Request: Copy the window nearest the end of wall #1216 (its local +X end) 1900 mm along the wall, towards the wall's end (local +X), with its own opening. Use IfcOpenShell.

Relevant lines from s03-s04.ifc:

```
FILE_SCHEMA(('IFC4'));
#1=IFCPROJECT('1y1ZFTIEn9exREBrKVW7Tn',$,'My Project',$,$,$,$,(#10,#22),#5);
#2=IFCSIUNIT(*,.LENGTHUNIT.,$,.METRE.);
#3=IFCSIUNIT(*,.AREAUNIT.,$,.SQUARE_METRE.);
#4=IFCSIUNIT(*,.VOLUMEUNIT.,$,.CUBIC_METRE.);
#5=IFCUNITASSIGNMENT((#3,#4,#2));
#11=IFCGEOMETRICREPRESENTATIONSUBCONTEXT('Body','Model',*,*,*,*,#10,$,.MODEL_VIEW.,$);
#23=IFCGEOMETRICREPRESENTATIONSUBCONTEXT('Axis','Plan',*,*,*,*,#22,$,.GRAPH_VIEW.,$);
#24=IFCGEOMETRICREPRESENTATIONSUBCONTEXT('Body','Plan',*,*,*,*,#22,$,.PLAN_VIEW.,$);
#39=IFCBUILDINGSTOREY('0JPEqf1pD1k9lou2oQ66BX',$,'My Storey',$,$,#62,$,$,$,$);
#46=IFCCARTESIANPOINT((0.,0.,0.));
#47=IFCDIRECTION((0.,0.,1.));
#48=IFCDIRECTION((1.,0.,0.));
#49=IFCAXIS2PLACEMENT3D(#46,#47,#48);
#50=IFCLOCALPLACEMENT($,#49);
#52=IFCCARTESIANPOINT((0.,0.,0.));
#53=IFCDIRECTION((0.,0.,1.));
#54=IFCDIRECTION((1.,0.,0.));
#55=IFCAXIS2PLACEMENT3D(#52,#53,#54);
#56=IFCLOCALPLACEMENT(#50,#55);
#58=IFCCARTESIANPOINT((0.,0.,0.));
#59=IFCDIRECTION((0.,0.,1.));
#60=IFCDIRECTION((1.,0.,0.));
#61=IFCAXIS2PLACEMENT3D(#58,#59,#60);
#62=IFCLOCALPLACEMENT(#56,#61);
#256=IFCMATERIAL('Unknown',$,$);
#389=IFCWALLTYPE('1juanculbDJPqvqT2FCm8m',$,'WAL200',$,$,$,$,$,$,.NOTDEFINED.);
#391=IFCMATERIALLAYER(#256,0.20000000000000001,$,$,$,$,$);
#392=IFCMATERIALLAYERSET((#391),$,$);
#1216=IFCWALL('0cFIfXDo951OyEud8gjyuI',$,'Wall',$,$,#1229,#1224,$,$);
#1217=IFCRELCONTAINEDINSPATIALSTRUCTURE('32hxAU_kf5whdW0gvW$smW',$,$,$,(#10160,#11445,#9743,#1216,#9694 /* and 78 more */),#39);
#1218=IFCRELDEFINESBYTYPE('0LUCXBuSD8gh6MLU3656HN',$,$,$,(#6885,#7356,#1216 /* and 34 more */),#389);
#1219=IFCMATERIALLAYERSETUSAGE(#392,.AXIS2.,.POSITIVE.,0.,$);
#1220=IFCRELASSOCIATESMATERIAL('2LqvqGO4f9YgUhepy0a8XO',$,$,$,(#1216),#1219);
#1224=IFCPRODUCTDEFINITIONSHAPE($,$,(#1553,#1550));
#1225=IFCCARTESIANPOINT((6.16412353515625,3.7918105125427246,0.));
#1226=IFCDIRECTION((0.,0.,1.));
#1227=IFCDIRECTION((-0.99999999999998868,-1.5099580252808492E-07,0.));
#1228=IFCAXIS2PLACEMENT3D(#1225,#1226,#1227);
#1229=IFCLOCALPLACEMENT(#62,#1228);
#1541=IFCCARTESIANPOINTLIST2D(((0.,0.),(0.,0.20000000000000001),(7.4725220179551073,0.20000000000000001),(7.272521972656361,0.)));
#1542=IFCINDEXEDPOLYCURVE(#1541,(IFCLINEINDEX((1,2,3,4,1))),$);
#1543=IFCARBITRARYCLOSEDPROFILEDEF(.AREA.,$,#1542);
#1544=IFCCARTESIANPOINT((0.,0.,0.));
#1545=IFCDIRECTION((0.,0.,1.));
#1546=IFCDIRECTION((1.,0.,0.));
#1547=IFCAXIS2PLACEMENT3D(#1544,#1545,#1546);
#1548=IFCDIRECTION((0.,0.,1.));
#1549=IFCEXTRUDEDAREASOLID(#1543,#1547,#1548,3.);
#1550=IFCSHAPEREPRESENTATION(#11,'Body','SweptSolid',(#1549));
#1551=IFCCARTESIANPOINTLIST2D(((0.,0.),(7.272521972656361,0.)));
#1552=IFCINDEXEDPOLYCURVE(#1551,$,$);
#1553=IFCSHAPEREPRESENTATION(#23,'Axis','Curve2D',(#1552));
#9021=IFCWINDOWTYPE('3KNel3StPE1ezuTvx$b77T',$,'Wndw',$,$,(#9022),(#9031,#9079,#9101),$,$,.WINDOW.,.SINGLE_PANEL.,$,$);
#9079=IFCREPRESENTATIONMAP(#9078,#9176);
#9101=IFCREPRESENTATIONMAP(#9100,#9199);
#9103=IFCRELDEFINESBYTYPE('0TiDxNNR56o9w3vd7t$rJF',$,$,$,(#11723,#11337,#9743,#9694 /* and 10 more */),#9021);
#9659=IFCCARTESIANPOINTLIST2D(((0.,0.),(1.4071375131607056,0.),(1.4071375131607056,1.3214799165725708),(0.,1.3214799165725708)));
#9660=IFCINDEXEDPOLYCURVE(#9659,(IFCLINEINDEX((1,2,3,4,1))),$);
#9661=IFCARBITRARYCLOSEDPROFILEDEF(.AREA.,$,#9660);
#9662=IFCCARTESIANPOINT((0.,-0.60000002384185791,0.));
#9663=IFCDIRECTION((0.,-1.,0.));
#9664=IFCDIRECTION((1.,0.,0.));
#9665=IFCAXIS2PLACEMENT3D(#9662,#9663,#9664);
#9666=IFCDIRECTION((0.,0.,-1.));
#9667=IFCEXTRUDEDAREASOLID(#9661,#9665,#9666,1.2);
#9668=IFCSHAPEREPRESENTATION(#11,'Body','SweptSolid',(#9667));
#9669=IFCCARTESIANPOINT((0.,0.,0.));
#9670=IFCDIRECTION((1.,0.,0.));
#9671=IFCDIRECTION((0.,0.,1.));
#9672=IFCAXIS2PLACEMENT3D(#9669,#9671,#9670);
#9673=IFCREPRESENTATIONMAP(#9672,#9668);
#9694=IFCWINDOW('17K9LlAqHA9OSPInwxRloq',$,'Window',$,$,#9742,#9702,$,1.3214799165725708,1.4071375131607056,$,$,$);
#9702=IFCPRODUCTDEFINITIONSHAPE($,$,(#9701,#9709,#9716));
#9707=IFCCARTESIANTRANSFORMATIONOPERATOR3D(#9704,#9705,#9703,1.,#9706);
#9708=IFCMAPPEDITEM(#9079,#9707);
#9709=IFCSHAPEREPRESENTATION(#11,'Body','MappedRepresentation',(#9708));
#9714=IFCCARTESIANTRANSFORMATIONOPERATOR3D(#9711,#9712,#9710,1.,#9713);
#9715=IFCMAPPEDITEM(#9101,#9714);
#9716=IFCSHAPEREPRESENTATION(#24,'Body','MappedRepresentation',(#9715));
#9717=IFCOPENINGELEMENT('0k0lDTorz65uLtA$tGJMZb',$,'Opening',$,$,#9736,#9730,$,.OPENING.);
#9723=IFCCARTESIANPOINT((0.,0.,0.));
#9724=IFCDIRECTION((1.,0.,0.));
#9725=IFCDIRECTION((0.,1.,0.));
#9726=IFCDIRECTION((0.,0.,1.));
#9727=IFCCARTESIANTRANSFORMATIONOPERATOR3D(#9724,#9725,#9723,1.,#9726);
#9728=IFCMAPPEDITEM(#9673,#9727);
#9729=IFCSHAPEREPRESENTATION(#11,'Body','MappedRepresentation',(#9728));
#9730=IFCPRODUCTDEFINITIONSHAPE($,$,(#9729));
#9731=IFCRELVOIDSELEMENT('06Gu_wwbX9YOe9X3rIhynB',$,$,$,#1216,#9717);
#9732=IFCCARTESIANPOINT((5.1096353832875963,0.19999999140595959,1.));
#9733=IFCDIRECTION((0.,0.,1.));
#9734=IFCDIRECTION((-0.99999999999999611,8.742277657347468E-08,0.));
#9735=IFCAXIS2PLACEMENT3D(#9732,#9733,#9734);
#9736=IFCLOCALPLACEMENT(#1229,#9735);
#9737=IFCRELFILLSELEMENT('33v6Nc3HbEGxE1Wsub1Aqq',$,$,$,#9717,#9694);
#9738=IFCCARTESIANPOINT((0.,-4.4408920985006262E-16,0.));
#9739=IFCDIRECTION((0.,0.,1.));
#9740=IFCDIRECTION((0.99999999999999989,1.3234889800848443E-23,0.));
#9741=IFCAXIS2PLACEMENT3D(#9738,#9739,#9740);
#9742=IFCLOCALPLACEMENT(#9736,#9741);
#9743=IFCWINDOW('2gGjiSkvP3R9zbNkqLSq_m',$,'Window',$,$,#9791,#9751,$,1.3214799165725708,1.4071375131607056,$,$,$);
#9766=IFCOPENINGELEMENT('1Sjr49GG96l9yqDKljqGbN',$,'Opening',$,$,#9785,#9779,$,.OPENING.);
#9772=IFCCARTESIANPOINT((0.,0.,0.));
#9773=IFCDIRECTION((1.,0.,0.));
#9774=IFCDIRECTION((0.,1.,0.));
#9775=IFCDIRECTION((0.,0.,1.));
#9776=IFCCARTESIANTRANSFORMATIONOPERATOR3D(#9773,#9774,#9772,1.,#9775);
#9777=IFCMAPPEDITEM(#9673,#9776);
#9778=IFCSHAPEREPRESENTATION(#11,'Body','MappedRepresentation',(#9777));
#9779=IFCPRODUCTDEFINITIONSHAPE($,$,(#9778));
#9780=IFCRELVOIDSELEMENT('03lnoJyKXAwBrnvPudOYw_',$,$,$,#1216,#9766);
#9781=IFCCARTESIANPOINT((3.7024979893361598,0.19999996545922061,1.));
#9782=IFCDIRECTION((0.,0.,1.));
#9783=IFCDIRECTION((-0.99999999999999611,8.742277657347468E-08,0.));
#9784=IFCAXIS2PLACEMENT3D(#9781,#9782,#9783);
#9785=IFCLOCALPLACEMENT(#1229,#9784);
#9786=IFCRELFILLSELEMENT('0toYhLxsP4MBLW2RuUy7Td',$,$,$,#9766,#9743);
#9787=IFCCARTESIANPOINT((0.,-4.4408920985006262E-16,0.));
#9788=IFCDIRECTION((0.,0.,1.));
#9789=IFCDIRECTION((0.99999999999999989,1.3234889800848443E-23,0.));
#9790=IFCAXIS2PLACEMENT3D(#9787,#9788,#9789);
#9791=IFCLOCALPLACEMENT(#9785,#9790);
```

```python
import ifcopenshell
import ifcopenshell.api.feature
import ifcopenshell.api.geometry
import ifcopenshell.api.root
import ifcopenshell.geom
import ifcopenshell.util.element
import ifcopenshell.util.placement
import ifcopenshell.util.shape
import ifcopenshell.util.unit

model = ifcopenshell.open("s03-s04.ifc")
unit_scale = ifcopenshell.util.unit.calculate_unit_scale(model)
settings = ifcopenshell.geom.settings()


def volume(element):
    """Net volume in cubic metres, openings subtracted."""
    shape = ifcopenshell.geom.create_shape(settings, element)
    return ifcopenshell.util.shape.get_volume(shape.geometry)


window = model.by_guid("17K9LlAqHA9OSPInwxRloq")
opening = window.FillsVoids[0].RelatingOpeningElement
wall = opening.VoidsElements[0].RelatingBuildingElement
before = volume(wall)
shift = ifcopenshell.util.placement.get_local_placement(wall.ObjectPlacement)[:3, 0] * 1.9 / unit_scale

# copy_class copies the void relationship, type, container and properties, but no geometry.
new_opening = ifcopenshell.api.root.copy_class(model, product=opening)
new_opening.Representation = ifcopenshell.util.element.copy_deep(
    model, opening.Representation, exclude=["IfcGeometricRepresentationContext", "IfcRepresentationMap"]
)
new_window = ifcopenshell.api.root.copy_class(model, product=window)
new_window.Representation = ifcopenshell.util.element.copy_deep(
    model, window.Representation, exclude=["IfcGeometricRepresentationContext", "IfcRepresentationMap"]
)
ifcopenshell.api.feature.add_filling(model, opening=new_opening, element=new_window)

for old, new in ((opening, new_opening), (window, new_window)):
    matrix = ifcopenshell.util.placement.get_local_placement(old.ObjectPlacement)
    matrix[:3, 3] += shift
    ifcopenshell.api.geometry.edit_object_placement(model, product=new, matrix=matrix, is_si=False)

after = volume(wall)

print(f"wall volume {before:.3f} -> {after:.3f} m3")

model.write("s03-s04_v2.ifc")
```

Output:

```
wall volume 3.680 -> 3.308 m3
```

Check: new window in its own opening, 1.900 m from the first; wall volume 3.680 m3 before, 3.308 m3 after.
